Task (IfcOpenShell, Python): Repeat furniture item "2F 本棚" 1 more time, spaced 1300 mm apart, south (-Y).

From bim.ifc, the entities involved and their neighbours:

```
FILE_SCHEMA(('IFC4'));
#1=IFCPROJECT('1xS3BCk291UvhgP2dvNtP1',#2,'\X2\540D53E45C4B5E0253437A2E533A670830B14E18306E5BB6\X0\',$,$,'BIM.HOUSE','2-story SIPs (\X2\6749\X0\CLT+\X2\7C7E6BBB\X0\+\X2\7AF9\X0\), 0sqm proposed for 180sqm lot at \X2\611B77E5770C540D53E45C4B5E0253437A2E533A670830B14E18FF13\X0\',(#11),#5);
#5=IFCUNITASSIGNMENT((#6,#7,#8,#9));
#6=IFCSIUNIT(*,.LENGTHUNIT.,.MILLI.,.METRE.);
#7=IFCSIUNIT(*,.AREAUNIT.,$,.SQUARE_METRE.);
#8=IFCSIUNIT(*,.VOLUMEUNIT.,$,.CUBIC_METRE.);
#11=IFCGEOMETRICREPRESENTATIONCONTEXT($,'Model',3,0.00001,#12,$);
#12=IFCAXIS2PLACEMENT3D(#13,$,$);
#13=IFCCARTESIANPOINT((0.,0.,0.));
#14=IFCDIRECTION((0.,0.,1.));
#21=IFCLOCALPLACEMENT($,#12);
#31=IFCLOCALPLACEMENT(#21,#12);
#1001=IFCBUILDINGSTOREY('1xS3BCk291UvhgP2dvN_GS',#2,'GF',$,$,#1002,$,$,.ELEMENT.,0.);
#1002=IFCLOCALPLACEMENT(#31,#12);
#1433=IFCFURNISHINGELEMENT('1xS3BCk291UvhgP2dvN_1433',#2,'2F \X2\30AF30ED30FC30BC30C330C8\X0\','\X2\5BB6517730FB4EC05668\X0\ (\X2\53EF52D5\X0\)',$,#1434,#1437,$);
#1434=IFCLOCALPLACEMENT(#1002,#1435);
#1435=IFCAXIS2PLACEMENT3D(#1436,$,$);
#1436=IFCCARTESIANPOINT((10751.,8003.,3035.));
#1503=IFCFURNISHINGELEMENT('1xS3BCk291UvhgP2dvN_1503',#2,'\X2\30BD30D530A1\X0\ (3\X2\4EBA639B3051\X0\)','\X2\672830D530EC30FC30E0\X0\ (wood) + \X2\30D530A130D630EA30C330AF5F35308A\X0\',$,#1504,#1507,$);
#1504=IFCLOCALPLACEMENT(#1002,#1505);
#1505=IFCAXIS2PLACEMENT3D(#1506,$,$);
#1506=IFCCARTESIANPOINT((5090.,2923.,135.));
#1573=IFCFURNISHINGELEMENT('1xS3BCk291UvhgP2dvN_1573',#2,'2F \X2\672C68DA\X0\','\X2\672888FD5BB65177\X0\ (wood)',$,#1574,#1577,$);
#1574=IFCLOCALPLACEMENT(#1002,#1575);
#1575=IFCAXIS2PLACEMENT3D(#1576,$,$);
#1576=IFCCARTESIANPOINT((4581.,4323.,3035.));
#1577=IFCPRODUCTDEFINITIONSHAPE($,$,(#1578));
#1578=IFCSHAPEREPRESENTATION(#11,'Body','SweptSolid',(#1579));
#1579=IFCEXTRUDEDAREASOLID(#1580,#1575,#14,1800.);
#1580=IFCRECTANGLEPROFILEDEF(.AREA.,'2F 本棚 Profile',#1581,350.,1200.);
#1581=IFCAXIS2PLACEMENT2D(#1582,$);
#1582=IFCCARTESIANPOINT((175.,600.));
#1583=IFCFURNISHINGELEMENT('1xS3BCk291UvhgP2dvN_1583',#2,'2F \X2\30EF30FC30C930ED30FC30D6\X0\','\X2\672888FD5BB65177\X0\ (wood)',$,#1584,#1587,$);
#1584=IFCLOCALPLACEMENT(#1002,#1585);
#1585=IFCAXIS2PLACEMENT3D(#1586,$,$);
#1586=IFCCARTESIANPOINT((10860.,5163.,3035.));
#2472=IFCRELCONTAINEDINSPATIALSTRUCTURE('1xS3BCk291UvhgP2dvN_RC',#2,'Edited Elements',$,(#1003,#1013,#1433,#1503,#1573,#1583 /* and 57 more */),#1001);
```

```python
import numpy as np
import ifcopenshell
import ifcopenshell.api.geometry
import ifcopenshell.api.root
import ifcopenshell.util.element
import ifcopenshell.util.placement
import ifcopenshell.util.unit

model = ifcopenshell.open("bim.ifc")
unit_scale = ifcopenshell.util.unit.calculate_unit_scale(model)


def reuse_history(source, copy):
    """copy_class also copies each property set's owner history, people and application; keep the originals."""
    for rel in copy.IsDefinedBy:
        if rel.is_a("IfcRelDefinesByProperties") and (history := rel.RelatingPropertyDefinition.OwnerHistory):
            rel.RelatingPropertyDefinition.OwnerHistory = source.OwnerHistory
            ifcopenshell.util.element.remove_deep2(model, history)


source = model.by_guid("1xS3BCk291UvhgP2dvN_1573")
base = ifcopenshell.util.placement.get_local_placement(source.ObjectPlacement)
step = np.array([0.0, -1.0, 0.0]) * 1.3 / unit_scale

for i in range(1, 2):
    copy = ifcopenshell.api.root.copy_class(model, product=source)
    copy.Representation = ifcopenshell.util.element.copy_deep(
        model, source.Representation, exclude=["IfcGeometricRepresentationContext", "IfcRepresentationMap"]
    )
    reuse_history(source, copy)
    matrix = base.copy()
    matrix[:3, 3] += i * step
    print("added at", matrix[:3, 3].round(3) + 0.0)
    ifcopenshell.api.geometry.edit_object_placement(model, product=copy, matrix=matrix, is_si=False)

model.write("bim-out.ifc")
```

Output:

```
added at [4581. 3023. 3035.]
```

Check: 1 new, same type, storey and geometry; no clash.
